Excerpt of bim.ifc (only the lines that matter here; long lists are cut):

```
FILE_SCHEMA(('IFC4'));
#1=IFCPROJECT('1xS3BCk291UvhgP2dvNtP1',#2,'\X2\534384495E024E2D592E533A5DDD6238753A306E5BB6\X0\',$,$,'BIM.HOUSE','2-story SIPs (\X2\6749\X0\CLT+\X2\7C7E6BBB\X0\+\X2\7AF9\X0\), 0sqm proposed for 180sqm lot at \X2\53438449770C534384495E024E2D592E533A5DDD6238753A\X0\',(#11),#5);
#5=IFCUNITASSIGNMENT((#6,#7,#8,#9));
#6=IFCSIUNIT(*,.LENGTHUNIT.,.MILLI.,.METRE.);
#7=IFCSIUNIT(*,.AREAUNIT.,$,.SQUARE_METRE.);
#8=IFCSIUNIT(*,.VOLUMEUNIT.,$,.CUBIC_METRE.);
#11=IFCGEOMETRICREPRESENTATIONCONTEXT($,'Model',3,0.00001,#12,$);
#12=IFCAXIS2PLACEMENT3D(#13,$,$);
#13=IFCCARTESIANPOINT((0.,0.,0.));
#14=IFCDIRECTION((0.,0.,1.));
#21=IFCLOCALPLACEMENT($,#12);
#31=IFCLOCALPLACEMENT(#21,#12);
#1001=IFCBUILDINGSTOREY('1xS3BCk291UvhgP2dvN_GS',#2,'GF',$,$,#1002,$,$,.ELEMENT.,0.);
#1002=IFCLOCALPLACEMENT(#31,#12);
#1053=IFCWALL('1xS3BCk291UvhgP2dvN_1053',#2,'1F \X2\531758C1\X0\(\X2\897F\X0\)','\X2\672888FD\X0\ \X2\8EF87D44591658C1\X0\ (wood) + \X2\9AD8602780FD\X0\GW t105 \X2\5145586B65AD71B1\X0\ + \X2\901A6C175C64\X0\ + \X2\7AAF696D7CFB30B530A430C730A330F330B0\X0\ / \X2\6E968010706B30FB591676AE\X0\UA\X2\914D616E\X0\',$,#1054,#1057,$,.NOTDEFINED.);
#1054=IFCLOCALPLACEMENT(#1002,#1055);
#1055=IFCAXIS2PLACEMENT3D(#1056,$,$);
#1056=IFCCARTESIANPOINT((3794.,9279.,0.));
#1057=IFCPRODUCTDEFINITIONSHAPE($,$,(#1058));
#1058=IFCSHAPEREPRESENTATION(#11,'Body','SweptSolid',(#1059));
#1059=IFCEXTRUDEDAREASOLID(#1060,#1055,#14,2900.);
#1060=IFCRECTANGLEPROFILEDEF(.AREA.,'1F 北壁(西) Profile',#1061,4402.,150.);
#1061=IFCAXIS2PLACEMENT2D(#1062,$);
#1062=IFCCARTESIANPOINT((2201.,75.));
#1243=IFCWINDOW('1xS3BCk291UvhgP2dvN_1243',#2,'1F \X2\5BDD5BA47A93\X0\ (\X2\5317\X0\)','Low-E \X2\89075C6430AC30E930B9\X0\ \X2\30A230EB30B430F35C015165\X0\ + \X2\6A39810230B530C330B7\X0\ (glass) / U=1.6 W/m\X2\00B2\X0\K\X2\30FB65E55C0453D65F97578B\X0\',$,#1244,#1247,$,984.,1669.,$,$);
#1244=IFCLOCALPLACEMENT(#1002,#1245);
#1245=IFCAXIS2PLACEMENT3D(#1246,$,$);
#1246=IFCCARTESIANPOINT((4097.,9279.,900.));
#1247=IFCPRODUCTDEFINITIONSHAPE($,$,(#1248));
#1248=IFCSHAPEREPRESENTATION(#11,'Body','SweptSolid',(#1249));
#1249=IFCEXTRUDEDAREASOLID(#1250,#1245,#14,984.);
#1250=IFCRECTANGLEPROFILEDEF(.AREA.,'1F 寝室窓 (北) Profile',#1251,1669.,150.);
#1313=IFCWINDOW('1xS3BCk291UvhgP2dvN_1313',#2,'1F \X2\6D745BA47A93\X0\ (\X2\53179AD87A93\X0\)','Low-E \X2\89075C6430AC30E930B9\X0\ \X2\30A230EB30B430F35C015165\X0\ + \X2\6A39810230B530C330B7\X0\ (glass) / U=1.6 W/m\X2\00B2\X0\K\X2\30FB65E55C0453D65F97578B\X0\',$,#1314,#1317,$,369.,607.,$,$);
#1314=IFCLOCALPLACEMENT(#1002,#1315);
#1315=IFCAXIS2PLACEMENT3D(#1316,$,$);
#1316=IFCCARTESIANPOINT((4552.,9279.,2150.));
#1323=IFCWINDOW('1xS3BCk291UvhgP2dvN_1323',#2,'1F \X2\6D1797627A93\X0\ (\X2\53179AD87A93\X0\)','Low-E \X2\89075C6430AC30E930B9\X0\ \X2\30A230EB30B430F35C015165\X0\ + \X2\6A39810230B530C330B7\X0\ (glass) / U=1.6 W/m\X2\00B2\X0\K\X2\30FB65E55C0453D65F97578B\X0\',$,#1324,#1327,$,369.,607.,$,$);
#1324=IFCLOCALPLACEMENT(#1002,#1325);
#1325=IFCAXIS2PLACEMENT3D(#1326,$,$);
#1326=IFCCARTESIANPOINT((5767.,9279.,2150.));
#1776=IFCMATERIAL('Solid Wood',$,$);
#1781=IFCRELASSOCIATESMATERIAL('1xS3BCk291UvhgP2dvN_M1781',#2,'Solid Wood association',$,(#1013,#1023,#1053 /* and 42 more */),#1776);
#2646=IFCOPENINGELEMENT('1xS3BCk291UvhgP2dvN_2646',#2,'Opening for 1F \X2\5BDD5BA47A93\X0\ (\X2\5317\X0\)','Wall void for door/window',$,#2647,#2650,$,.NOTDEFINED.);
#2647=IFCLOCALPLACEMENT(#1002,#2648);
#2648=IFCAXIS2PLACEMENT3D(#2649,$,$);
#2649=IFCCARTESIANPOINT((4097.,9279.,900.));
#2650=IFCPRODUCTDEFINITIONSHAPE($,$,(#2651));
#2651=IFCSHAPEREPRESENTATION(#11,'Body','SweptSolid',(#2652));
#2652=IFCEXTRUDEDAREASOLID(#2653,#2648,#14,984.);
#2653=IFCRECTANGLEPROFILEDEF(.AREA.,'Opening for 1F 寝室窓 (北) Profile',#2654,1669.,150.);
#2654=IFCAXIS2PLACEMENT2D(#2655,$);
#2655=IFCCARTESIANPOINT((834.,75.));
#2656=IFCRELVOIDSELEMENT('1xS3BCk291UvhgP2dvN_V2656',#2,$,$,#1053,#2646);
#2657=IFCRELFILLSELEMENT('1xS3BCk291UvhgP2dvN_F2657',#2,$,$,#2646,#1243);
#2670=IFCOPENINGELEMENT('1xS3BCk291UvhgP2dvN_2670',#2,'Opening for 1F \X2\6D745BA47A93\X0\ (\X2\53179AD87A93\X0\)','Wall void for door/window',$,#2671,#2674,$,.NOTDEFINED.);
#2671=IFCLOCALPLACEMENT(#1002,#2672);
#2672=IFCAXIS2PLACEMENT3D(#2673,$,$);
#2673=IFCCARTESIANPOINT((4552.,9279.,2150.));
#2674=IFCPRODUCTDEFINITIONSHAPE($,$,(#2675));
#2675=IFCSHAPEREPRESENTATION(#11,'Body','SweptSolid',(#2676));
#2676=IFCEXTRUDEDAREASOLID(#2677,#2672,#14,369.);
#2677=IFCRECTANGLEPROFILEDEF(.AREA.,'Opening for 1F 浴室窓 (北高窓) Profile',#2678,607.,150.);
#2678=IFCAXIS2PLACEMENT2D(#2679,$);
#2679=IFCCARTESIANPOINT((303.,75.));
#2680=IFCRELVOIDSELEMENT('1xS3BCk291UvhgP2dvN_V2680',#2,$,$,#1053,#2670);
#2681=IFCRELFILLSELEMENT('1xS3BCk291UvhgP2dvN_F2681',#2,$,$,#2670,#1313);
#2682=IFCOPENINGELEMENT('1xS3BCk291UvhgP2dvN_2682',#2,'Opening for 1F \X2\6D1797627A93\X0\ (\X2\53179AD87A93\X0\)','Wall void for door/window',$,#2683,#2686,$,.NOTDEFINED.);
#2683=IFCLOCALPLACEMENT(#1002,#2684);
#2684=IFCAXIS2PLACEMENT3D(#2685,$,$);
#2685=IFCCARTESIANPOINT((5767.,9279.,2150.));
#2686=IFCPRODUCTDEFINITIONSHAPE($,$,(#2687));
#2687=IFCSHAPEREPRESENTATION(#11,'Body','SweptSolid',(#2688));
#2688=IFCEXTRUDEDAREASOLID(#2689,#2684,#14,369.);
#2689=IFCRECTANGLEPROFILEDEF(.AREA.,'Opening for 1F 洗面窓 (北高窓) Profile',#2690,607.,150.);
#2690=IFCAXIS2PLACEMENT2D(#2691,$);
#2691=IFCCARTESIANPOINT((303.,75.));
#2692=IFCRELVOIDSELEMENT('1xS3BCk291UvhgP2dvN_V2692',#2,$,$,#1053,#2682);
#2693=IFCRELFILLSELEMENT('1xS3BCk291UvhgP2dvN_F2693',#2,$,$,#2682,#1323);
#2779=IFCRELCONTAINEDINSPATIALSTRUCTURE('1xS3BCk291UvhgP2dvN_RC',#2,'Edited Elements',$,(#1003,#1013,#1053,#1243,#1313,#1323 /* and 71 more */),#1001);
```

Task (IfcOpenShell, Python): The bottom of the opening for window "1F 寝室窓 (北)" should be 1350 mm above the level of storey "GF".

```python
import numpy as np
import ifcopenshell
import ifcopenshell.api.geometry
import ifcopenshell.geom
import ifcopenshell.util.element
import ifcopenshell.util.placement
import ifcopenshell.util.shape
import ifcopenshell.util.unit

model = ifcopenshell.open("bim.ifc")
unit_scale = ifcopenshell.util.unit.calculate_unit_scale(model)

window = model.by_guid("1xS3BCk291UvhgP2dvN_1243")
opening = window.FillsVoids[0].RelatingOpeningElement
storey = ifcopenshell.util.element.get_container(window, ifc_class="IfcBuildingStorey")
level = ifcopenshell.util.placement.get_local_placement(storey.ObjectPlacement)[2, 3]

# The opening's origin need not be at the sill, so measure its lowest point.
shape = ifcopenshell.geom.create_shape(ifcopenshell.geom.settings(), opening)
bottom = ifcopenshell.util.shape.get_shape_bottom_elevation(shape, shape.geometry) / unit_scale
dz = level + 1350.0 - bottom

shift = np.array([0.0, 0.0, dz])
# The window is not placed relative to its opening, so move both.
for product in (opening, window):
    matrix = ifcopenshell.util.placement.get_local_placement(product.ObjectPlacement)
    matrix[:3, 3] += shift
    ifcopenshell.api.geometry.edit_object_placement(model, product=product, matrix=matrix, is_si=False)

print(f"moved by {dz * unit_scale:+.3f} m")

model.write("bim_v2.ifc")
```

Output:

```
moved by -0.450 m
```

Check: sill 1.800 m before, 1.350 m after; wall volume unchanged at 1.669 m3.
